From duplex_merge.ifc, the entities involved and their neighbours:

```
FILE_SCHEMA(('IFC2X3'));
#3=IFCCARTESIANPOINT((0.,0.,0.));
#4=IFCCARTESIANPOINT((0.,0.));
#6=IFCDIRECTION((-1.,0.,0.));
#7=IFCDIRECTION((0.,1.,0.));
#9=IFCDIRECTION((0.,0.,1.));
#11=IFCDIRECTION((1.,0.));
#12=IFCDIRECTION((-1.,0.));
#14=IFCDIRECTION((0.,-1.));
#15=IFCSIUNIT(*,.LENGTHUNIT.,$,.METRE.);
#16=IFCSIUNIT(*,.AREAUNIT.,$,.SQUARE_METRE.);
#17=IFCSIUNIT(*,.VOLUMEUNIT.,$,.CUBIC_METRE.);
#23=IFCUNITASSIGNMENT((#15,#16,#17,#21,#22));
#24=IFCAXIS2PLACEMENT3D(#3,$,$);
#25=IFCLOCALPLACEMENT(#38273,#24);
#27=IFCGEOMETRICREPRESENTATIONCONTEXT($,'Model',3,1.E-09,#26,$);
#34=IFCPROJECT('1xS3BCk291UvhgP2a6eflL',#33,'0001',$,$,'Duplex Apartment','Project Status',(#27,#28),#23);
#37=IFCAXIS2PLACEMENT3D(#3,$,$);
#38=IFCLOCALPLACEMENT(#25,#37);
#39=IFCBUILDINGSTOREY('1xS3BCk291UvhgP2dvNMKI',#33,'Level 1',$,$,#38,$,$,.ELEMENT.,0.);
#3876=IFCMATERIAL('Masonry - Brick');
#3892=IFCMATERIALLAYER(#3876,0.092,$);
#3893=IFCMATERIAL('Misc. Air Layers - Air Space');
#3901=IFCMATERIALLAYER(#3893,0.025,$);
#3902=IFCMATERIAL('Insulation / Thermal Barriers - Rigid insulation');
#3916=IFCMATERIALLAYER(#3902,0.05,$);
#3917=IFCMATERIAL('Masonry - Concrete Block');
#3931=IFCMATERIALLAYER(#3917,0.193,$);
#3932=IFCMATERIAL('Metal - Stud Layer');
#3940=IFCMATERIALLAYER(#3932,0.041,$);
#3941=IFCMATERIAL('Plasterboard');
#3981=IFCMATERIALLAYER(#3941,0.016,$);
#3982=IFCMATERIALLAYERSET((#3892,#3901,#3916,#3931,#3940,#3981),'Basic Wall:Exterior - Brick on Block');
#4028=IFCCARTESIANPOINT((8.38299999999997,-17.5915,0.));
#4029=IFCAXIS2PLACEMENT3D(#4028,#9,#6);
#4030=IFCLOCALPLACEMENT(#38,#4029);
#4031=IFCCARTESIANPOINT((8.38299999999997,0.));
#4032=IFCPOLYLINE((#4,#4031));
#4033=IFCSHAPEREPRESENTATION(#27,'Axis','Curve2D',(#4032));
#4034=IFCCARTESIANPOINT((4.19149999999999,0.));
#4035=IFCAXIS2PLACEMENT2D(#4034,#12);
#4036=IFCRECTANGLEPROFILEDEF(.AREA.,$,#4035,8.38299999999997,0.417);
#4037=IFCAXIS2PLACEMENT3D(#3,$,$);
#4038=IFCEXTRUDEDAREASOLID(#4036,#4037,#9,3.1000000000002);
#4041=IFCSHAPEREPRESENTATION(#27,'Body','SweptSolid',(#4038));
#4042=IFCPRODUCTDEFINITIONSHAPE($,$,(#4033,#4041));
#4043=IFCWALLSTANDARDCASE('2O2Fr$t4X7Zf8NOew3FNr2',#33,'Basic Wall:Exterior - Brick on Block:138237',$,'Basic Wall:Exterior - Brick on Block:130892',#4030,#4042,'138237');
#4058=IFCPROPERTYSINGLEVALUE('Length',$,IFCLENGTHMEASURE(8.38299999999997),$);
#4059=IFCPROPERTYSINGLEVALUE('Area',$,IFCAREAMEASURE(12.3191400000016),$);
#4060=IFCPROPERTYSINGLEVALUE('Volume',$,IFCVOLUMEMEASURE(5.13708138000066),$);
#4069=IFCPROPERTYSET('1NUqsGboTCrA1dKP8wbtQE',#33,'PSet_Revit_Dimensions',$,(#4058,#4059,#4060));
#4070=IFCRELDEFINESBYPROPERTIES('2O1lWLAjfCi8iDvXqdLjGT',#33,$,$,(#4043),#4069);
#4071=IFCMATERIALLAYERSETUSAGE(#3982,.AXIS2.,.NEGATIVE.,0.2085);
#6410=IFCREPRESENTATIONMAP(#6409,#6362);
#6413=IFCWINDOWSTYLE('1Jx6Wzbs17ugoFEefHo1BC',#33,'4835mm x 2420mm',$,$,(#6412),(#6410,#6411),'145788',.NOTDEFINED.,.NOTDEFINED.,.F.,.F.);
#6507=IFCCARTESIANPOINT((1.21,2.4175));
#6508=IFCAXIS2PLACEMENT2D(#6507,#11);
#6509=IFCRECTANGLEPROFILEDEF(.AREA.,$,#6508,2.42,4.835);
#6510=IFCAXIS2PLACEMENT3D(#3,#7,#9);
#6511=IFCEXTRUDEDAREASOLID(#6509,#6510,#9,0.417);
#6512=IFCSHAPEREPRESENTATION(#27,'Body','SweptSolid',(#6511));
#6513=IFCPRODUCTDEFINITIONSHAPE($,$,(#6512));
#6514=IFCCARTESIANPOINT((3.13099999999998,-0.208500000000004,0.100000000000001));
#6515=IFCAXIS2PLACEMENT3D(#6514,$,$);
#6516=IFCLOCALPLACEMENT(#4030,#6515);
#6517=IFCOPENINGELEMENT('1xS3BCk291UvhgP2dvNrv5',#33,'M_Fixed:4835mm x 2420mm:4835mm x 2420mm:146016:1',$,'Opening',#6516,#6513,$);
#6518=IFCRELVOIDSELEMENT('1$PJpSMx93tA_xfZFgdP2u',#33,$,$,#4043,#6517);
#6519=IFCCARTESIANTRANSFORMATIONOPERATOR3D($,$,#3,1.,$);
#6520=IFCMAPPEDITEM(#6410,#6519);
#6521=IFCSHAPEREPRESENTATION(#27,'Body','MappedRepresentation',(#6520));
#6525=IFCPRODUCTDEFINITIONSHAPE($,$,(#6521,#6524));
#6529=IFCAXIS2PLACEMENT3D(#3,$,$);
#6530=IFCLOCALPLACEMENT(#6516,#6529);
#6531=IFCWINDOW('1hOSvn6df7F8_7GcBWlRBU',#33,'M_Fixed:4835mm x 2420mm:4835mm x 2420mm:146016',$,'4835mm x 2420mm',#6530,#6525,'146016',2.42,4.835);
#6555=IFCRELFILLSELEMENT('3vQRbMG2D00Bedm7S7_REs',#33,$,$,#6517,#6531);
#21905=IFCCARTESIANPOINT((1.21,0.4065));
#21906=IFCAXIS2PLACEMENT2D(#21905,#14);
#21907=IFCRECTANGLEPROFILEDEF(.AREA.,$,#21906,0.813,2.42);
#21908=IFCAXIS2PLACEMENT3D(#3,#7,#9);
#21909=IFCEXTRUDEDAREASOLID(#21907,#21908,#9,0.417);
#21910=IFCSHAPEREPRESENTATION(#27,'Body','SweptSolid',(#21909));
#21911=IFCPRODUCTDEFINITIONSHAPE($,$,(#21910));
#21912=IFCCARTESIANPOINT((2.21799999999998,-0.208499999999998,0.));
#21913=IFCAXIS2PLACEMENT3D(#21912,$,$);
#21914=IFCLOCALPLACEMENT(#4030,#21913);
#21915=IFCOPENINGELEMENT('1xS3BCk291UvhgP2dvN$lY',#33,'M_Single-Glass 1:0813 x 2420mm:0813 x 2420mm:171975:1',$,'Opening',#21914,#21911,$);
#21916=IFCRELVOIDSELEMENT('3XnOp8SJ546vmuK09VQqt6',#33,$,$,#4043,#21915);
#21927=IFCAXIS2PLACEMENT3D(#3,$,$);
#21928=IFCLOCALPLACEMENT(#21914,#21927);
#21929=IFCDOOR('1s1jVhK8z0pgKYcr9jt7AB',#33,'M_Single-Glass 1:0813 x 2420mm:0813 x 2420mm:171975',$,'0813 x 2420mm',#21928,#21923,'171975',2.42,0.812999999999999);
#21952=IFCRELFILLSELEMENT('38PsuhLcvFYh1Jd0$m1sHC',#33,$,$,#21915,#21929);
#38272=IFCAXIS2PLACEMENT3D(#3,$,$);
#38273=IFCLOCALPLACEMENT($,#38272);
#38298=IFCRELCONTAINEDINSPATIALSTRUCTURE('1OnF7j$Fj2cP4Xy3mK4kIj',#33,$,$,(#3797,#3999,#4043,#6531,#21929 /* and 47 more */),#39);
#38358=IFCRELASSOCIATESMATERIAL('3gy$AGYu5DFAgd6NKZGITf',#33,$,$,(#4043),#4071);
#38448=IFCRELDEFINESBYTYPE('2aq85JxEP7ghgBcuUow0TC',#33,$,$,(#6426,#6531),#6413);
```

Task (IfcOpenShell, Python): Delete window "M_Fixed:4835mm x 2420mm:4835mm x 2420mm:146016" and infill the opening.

```python
import ifcopenshell
import ifcopenshell.api.feature
import ifcopenshell.api.pset
import ifcopenshell.api.root
import ifcopenshell.geom
import ifcopenshell.util.element
import ifcopenshell.util.shape
import ifcopenshell.util.unit

model = ifcopenshell.open("duplex_merge.ifc")
area_scale = ifcopenshell.util.unit.calculate_unit_scale(model, "AREAUNIT")
volume_scale = ifcopenshell.util.unit.calculate_unit_scale(model, "VOLUMEUNIT")
settings = ifcopenshell.geom.settings()


def volume(element):
    """Net volume in cubic metres, openings subtracted."""
    shape = ifcopenshell.geom.create_shape(settings, element)
    return ifcopenshell.util.shape.get_volume(shape.geometry)


window = model.by_id(6531)
opening = window.FillsVoids[0].RelatingOpeningElement
wall = opening.VoidsElements[0].RelatingBuildingElement
before = volume(wall)

ifcopenshell.api.root.remove_product(model, product=window)
ifcopenshell.api.feature.remove_feature(model, feature=opening)

after = volume(wall)
thickness = 0.417  # wall thickness in metres

# Update the wall's stored quantities.
pset = model.by_id(ifcopenshell.util.element.get_pset(wall, "PSet_Revit_Dimensions", should_inherit=False)["id"])
ifcopenshell.api.pset.edit_pset(model, pset=pset, properties={
    "Area": model.create_entity("IfcAreaMeasure", after / thickness / area_scale),
    "Volume": model.create_entity("IfcVolumeMeasure", after / volume_scale),
})

print(f"wall volume {before:.3f} -> {after:.3f} m3")

model.write("duplex_merge_rev.ifc")
```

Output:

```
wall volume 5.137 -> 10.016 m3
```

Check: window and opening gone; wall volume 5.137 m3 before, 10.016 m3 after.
